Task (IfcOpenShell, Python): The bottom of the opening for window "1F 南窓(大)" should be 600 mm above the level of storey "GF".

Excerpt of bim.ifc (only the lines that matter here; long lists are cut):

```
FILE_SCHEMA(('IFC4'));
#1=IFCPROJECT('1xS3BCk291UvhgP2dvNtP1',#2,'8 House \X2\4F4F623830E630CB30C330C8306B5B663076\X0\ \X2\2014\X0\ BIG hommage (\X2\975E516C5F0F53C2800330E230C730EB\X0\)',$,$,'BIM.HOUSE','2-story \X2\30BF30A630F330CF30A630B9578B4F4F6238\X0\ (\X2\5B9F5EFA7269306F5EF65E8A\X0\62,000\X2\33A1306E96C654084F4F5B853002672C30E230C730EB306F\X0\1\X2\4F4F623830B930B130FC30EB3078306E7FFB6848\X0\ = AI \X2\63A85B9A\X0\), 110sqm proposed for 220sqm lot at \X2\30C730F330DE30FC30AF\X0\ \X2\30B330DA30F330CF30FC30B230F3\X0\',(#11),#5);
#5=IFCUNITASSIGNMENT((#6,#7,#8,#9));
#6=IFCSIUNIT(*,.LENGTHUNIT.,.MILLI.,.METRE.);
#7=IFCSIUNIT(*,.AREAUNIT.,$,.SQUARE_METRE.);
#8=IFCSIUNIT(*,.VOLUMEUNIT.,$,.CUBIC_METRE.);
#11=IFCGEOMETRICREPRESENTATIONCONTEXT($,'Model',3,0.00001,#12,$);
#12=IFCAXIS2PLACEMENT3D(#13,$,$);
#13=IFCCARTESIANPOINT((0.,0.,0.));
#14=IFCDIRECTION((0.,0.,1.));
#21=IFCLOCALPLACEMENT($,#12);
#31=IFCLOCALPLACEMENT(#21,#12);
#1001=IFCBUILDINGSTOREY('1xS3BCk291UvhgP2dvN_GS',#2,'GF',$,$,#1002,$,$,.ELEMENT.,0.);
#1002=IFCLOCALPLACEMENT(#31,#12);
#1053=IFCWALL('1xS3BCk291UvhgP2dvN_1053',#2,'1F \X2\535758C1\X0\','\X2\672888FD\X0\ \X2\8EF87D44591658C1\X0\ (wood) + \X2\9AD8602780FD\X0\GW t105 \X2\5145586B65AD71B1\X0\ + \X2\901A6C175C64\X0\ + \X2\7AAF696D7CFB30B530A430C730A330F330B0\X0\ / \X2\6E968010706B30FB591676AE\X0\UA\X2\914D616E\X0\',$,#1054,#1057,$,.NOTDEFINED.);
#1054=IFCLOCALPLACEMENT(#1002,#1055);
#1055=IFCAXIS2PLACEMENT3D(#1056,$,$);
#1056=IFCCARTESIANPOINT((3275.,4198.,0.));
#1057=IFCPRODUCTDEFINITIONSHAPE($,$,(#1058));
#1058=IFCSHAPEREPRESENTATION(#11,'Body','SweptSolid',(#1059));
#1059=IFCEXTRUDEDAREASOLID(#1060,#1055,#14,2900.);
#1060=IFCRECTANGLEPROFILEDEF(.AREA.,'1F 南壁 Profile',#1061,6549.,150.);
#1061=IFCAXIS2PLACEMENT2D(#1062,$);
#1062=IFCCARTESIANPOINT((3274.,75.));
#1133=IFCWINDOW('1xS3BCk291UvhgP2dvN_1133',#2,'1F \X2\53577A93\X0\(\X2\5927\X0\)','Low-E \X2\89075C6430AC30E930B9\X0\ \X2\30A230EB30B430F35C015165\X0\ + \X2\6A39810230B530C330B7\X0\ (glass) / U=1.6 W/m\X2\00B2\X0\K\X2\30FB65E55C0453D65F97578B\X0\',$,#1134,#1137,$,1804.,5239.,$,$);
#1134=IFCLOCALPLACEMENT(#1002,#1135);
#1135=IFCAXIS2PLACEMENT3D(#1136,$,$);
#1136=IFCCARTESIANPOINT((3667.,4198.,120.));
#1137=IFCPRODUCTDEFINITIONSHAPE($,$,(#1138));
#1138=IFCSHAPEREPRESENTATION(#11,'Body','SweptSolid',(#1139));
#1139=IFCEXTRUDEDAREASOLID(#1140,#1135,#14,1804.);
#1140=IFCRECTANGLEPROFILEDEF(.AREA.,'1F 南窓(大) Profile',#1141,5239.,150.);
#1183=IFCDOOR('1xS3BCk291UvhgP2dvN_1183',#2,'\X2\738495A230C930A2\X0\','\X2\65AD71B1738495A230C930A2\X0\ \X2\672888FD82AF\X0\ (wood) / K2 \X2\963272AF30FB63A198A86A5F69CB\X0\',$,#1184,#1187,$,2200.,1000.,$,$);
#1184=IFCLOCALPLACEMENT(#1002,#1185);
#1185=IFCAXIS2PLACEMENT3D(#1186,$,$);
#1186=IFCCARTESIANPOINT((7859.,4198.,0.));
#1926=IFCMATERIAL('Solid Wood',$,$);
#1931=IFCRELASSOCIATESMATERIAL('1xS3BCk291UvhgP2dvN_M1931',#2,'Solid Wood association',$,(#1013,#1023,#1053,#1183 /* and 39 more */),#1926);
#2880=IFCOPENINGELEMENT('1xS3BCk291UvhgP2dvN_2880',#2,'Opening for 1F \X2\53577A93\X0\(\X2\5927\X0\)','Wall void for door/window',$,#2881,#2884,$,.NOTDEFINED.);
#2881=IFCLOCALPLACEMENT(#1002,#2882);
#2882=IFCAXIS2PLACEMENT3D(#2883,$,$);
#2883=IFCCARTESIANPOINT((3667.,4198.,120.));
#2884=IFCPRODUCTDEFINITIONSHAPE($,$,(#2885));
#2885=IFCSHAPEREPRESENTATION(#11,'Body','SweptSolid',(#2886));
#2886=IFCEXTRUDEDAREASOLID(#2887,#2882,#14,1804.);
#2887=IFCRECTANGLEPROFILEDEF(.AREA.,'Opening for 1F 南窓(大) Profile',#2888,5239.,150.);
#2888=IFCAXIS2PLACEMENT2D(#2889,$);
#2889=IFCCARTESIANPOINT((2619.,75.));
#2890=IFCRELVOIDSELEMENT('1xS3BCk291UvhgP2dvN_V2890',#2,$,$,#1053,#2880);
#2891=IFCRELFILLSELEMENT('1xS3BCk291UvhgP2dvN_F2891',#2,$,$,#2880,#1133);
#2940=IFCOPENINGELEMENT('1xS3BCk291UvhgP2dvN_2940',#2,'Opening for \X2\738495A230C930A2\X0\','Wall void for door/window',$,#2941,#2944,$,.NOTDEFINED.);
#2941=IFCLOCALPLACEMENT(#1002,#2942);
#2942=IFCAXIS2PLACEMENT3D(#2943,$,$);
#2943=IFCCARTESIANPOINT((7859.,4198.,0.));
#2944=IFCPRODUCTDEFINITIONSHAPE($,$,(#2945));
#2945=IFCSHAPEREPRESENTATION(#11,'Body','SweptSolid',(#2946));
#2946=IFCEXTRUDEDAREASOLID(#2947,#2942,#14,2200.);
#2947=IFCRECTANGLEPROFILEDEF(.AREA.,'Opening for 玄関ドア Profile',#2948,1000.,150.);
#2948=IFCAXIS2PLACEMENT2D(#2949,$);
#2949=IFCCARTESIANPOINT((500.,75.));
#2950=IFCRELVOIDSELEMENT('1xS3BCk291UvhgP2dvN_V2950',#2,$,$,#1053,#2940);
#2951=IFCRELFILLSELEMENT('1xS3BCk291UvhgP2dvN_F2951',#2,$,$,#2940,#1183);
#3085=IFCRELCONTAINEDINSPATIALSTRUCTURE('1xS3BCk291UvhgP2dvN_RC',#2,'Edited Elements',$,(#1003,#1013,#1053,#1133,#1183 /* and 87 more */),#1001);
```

```python
import numpy as np
import ifcopenshell
import ifcopenshell.api.geometry
import ifcopenshell.geom
import ifcopenshell.util.element
import ifcopenshell.util.placement
import ifcopenshell.util.shape
import ifcopenshell.util.unit

model = ifcopenshell.open("bim.ifc")
unit_scale = ifcopenshell.util.unit.calculate_unit_scale(model)

window = model.by_guid("1xS3BCk291UvhgP2dvN_1133")
opening = window.FillsVoids[0].RelatingOpeningElement
storey = ifcopenshell.util.element.get_container(window, ifc_class="IfcBuildingStorey")
level = ifcopenshell.util.placement.get_local_placement(storey.ObjectPlacement)[2, 3]

# The opening's origin need not be at the sill, so measure its lowest point.
shape = ifcopenshell.geom.create_shape(ifcopenshell.geom.settings(), opening)
bottom = ifcopenshell.util.shape.get_shape_bottom_elevation(shape, shape.geometry) / unit_scale
dz = level + 0.6 / unit_scale - bottom

shift = np.array([0.0, 0.0, dz])
# The window is not placed relative to its opening, so move both.
for product in (opening, window):
    matrix = ifcopenshell.util.placement.get_local_placement(product.ObjectPlacement)
    matrix[:3, 3] += shift
    ifcopenshell.api.geometry.edit_object_placement(model, product=product, matrix=matrix, is_si=False)

print(f"moved by {dz * unit_scale:+.3f} m")

model.write("bim_edited.ifc")
```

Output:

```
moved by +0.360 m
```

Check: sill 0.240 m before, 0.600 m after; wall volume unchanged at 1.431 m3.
